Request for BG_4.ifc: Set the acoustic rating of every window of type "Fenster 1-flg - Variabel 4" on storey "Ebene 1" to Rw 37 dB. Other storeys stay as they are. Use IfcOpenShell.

First a look at what the model holds.

```python
import ifcopenshell
import ifcopenshell.util.element

model = ifcopenshell.open("BG_4.ifc")
print(model.schema)
storey = next(s for s in model.by_type("IfcBuildingStorey") if s.Name == "Ebene 1")
windows = [e for e in ifcopenshell.util.element.get_decomposition(storey) if e.is_a("IfcWindow")]
seen = {}
for e in windows:
    element_type = ifcopenshell.util.element.get_type(e)
    key = (element_type.Name if element_type != e and element_type else None, ifcopenshell.util.element.get_pset(e, "Pset_WindowCommon", "AcousticRating"))
    seen[key] = seen.get(key, 0) + 1
for (name, value), count in sorted(seen.items(), key=str):
    print(count, "x", name, "|", value)
```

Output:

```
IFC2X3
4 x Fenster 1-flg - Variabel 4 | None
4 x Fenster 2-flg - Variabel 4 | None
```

```python
import ifcopenshell
import ifcopenshell.api.pset
import ifcopenshell.util.element

model = ifcopenshell.open("BG_4.ifc")

storey = next(s for s in model.by_type("IfcBuildingStorey") if s.Name == "Ebene 1")
windows = [e for e in ifcopenshell.util.element.get_decomposition(storey) if e.is_a("IfcWindow")]

count = 0
for e in windows:
    element_type = ifcopenshell.util.element.get_type(e)
    if element_type in (None, e) or element_type.Name != "Fenster 1-flg - Variabel 4":
        continue
    # add_pset returns the element's existing set when there is one.
    pset = ifcopenshell.api.pset.add_pset(model, product=e, name="Pset_WindowCommon")
    ifcopenshell.api.pset.edit_pset(model, pset=pset, properties={"AcousticRating": "Rw 37 dB"})
    count += 1

print(count, "windows updated")

model.write("BG_4_updated.ifc")
```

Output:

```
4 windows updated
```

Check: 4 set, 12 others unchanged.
